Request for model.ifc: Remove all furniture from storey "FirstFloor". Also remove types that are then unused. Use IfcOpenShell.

First a look at what the model holds.

```python
import ifcopenshell
import ifcopenshell.util.element

model = ifcopenshell.open("model.ifc")
print(model.schema)
storey = next(s for s in model.by_type("IfcBuildingStorey") if s.Name == "FirstFloor")
furniture = [e for e in ifcopenshell.util.element.get_decomposition(storey) if e.is_a("IfcFurnishingElement")]
seen = {}
for e in furniture:
    element_type = ifcopenshell.util.element.get_type(e)
    name = element_type.Name if element_type not in (None, e) else None
    seen[name] = seen.get(name, 0) + 1
for name, count in sorted(seen.items(), key=str):
    print(count, "x", name)
```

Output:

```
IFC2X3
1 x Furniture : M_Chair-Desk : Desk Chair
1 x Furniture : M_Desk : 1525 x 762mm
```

```python
import ifcopenshell
import ifcopenshell.api.root
import ifcopenshell.util.element

model = ifcopenshell.open("model.ifc")

storey = next(s for s in model.by_type("IfcBuildingStorey") if s.Name == "FirstFloor")
furniture = [e for e in ifcopenshell.util.element.get_decomposition(storey) if e.is_a("IfcFurnishingElement")]
types = {ifcopenshell.util.element.get_type(e) for e in furniture} - {None, *furniture}

for e in furniture:
    ifcopenshell.api.root.remove_product(model, product=e)
print(len(furniture), "removed")

unused = [t for t in types if not ifcopenshell.util.element.get_types(t)]
for t in unused:
    ifcopenshell.api.root.remove_product(model, product=t)
print(len(unused), "unused types removed")

model.write("model_edited.ifc")
```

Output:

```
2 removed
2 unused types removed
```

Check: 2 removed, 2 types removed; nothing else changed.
